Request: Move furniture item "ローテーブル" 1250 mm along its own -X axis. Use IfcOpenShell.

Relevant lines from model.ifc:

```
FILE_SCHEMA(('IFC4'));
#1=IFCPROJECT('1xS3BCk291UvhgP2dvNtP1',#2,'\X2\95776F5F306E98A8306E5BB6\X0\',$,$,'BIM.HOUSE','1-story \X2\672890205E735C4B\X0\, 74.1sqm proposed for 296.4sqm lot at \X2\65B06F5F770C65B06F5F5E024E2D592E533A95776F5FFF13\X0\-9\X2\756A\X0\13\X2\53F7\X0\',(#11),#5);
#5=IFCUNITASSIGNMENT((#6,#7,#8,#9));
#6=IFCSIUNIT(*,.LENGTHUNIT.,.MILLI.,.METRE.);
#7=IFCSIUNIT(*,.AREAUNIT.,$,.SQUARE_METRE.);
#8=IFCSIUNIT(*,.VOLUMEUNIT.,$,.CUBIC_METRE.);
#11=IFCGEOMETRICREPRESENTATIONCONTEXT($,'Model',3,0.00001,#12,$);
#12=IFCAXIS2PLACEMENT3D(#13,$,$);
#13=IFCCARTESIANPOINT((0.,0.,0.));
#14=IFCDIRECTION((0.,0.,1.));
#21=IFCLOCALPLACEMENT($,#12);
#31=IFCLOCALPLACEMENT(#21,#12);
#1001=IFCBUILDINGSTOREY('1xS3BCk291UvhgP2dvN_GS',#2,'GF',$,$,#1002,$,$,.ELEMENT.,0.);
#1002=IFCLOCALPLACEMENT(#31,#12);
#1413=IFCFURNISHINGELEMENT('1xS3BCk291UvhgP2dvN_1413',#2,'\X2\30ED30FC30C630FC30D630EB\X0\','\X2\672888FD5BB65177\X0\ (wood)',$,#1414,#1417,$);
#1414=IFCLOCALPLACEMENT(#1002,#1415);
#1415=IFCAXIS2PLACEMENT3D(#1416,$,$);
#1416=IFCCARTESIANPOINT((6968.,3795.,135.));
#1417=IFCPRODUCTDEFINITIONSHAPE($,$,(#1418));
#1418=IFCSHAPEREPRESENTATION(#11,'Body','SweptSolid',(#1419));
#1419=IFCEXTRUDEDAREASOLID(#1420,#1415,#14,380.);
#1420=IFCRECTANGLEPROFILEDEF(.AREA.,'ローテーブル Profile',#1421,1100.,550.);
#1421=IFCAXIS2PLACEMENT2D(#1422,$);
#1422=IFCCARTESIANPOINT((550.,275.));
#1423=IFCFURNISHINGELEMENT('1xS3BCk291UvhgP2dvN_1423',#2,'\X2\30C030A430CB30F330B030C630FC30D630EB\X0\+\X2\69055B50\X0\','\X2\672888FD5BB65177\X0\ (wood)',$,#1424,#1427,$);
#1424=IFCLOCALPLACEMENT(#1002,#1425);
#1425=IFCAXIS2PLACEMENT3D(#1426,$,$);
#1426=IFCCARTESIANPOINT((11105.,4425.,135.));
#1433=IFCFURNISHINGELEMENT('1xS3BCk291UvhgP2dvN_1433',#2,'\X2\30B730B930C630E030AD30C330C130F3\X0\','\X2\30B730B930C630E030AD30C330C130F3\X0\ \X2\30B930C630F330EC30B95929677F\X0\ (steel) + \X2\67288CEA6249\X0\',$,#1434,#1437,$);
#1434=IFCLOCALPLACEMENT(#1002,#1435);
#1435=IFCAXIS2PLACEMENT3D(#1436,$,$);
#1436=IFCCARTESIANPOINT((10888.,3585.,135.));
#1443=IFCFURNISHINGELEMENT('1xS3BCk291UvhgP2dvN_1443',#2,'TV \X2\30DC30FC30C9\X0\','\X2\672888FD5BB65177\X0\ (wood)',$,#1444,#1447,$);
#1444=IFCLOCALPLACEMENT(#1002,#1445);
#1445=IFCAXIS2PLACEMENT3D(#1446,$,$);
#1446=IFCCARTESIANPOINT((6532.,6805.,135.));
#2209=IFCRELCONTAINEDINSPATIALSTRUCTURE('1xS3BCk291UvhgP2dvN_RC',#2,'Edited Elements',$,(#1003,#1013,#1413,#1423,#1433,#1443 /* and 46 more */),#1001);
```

```python
import ifcopenshell
import ifcopenshell.api.geometry
import ifcopenshell.util.placement

model = ifcopenshell.open("model.ifc")

item = model.by_id(1413)
matrix = ifcopenshell.util.placement.get_local_placement(item.ObjectPlacement)
matrix[:3, 3] -= matrix[:3, 0] * 1250.0
ifcopenshell.api.geometry.edit_object_placement(model, product=item, matrix=matrix, is_si=False)

print(ifcopenshell.util.placement.get_local_placement(item.ObjectPlacement).round(3) + 0.0)

model.write("model_v2.ifc")
```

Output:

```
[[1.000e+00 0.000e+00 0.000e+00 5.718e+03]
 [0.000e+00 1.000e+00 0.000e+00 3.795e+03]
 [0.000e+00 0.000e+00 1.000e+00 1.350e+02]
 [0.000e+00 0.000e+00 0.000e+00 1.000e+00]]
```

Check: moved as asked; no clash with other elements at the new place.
